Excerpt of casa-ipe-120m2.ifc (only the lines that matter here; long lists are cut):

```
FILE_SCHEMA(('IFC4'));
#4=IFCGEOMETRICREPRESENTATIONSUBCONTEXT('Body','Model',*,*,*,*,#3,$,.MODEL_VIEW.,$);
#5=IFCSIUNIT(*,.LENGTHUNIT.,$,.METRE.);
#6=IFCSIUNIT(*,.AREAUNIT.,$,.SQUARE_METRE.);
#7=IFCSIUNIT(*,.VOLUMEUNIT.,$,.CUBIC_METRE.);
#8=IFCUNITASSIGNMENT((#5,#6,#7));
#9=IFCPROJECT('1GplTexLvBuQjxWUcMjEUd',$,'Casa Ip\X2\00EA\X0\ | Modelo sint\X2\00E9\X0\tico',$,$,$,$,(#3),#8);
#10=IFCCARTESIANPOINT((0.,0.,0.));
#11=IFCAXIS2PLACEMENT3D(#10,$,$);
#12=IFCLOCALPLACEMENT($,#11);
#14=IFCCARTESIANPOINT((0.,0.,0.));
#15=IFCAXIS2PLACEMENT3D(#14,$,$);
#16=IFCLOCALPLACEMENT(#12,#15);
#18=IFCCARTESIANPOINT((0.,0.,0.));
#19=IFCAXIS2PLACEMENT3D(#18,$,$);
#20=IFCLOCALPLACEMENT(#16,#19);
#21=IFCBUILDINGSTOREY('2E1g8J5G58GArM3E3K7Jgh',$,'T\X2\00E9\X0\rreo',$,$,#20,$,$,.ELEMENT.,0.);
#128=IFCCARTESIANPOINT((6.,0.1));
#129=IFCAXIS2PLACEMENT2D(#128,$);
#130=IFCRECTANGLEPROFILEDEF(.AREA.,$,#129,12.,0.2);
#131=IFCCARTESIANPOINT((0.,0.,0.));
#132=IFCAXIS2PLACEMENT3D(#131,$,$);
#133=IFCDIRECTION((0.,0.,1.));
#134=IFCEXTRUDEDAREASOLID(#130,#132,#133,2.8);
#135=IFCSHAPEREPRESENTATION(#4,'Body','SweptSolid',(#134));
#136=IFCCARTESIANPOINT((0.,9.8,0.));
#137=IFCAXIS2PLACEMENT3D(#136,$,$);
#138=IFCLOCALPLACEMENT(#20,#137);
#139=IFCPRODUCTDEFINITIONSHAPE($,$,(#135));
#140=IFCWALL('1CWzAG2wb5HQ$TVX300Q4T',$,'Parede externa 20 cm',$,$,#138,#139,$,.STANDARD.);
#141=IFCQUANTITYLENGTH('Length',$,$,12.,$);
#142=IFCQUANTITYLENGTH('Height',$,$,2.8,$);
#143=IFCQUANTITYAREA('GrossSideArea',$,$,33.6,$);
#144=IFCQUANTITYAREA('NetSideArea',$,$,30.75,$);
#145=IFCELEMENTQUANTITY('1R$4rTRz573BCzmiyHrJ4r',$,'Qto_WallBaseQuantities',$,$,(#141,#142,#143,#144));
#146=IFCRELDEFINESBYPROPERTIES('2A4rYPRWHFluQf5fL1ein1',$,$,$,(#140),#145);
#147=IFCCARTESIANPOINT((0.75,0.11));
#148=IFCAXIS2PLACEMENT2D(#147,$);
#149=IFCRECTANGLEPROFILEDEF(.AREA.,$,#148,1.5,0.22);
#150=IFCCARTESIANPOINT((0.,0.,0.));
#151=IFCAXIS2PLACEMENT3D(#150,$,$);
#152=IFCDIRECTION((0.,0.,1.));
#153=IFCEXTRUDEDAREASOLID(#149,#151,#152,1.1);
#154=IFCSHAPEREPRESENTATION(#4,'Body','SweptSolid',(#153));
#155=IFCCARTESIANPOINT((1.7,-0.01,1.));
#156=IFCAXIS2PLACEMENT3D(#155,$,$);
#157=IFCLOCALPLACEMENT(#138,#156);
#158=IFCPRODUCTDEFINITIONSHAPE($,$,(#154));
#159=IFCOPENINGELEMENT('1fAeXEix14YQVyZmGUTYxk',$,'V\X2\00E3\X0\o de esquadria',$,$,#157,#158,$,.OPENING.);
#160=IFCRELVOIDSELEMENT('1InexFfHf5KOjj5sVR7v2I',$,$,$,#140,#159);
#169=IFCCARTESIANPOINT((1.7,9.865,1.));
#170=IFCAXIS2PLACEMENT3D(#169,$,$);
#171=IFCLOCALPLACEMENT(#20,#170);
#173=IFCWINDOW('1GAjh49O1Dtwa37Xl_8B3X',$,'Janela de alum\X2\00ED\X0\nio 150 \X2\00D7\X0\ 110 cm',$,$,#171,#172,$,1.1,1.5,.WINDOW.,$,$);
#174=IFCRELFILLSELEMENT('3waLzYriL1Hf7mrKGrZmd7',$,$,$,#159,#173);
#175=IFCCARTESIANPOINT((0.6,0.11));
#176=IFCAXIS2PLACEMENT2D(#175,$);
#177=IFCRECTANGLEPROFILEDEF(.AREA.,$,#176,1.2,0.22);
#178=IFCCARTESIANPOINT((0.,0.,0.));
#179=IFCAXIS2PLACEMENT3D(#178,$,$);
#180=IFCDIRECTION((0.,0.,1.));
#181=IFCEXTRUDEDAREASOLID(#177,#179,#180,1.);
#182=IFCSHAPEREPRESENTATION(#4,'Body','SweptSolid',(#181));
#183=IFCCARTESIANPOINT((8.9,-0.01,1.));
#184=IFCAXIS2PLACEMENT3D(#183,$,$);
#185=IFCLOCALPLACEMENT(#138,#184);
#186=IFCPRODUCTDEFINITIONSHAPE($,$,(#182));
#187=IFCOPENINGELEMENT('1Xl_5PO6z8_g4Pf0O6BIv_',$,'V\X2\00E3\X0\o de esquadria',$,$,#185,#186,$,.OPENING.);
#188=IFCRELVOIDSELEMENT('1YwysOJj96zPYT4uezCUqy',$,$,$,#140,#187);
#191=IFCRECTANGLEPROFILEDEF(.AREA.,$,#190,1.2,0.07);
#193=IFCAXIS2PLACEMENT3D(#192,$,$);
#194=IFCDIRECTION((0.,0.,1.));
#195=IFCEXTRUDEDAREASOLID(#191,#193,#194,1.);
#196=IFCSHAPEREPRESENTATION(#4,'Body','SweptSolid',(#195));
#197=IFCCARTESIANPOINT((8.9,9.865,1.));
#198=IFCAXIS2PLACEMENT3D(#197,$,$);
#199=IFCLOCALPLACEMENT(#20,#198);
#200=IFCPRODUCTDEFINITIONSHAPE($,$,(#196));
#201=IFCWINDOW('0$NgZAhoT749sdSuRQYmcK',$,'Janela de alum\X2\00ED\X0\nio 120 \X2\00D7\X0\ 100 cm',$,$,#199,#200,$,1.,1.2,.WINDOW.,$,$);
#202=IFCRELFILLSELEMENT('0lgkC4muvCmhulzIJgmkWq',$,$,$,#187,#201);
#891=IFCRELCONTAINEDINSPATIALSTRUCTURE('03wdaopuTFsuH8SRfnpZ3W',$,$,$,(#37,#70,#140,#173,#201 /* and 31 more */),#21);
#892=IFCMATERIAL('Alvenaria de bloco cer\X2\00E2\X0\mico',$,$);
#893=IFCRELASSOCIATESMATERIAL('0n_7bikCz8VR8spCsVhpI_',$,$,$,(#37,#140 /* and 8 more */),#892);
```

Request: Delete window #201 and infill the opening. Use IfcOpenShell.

```python
import ifcopenshell
import ifcopenshell.api.feature
import ifcopenshell.api.pset
import ifcopenshell.api.root
import ifcopenshell.geom
import ifcopenshell.util.element
import ifcopenshell.util.shape
import ifcopenshell.util.unit

model = ifcopenshell.open("casa-ipe-120m2.ifc")
area_scale = ifcopenshell.util.unit.calculate_unit_scale(model, "AREAUNIT")
settings = ifcopenshell.geom.settings()


def volume(element):
    """Net volume in cubic metres, openings subtracted."""
    shape = ifcopenshell.geom.create_shape(settings, element)
    return ifcopenshell.util.shape.get_volume(shape.geometry)


window = model.by_guid("0$NgZAhoT749sdSuRQYmcK")
opening = window.FillsVoids[0].RelatingOpeningElement
wall = opening.VoidsElements[0].RelatingBuildingElement
before = volume(wall)

ifcopenshell.api.root.remove_product(model, product=window)
ifcopenshell.api.feature.remove_feature(model, feature=opening)

after = volume(wall)
thickness = 0.2  # wall thickness in metres

# Update the wall's stored quantities.
qto = model.by_id(ifcopenshell.util.element.get_pset(wall, "Qto_WallBaseQuantities", should_inherit=False)["id"])
ifcopenshell.api.pset.edit_qto(model, qto=qto, properties={"NetSideArea": after / thickness / area_scale})

print(f"wall volume {before:.3f} -> {after:.3f} m3")

model.write("casa-ipe-120m2_updated.ifc")
```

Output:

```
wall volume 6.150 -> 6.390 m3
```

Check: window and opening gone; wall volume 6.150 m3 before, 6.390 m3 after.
